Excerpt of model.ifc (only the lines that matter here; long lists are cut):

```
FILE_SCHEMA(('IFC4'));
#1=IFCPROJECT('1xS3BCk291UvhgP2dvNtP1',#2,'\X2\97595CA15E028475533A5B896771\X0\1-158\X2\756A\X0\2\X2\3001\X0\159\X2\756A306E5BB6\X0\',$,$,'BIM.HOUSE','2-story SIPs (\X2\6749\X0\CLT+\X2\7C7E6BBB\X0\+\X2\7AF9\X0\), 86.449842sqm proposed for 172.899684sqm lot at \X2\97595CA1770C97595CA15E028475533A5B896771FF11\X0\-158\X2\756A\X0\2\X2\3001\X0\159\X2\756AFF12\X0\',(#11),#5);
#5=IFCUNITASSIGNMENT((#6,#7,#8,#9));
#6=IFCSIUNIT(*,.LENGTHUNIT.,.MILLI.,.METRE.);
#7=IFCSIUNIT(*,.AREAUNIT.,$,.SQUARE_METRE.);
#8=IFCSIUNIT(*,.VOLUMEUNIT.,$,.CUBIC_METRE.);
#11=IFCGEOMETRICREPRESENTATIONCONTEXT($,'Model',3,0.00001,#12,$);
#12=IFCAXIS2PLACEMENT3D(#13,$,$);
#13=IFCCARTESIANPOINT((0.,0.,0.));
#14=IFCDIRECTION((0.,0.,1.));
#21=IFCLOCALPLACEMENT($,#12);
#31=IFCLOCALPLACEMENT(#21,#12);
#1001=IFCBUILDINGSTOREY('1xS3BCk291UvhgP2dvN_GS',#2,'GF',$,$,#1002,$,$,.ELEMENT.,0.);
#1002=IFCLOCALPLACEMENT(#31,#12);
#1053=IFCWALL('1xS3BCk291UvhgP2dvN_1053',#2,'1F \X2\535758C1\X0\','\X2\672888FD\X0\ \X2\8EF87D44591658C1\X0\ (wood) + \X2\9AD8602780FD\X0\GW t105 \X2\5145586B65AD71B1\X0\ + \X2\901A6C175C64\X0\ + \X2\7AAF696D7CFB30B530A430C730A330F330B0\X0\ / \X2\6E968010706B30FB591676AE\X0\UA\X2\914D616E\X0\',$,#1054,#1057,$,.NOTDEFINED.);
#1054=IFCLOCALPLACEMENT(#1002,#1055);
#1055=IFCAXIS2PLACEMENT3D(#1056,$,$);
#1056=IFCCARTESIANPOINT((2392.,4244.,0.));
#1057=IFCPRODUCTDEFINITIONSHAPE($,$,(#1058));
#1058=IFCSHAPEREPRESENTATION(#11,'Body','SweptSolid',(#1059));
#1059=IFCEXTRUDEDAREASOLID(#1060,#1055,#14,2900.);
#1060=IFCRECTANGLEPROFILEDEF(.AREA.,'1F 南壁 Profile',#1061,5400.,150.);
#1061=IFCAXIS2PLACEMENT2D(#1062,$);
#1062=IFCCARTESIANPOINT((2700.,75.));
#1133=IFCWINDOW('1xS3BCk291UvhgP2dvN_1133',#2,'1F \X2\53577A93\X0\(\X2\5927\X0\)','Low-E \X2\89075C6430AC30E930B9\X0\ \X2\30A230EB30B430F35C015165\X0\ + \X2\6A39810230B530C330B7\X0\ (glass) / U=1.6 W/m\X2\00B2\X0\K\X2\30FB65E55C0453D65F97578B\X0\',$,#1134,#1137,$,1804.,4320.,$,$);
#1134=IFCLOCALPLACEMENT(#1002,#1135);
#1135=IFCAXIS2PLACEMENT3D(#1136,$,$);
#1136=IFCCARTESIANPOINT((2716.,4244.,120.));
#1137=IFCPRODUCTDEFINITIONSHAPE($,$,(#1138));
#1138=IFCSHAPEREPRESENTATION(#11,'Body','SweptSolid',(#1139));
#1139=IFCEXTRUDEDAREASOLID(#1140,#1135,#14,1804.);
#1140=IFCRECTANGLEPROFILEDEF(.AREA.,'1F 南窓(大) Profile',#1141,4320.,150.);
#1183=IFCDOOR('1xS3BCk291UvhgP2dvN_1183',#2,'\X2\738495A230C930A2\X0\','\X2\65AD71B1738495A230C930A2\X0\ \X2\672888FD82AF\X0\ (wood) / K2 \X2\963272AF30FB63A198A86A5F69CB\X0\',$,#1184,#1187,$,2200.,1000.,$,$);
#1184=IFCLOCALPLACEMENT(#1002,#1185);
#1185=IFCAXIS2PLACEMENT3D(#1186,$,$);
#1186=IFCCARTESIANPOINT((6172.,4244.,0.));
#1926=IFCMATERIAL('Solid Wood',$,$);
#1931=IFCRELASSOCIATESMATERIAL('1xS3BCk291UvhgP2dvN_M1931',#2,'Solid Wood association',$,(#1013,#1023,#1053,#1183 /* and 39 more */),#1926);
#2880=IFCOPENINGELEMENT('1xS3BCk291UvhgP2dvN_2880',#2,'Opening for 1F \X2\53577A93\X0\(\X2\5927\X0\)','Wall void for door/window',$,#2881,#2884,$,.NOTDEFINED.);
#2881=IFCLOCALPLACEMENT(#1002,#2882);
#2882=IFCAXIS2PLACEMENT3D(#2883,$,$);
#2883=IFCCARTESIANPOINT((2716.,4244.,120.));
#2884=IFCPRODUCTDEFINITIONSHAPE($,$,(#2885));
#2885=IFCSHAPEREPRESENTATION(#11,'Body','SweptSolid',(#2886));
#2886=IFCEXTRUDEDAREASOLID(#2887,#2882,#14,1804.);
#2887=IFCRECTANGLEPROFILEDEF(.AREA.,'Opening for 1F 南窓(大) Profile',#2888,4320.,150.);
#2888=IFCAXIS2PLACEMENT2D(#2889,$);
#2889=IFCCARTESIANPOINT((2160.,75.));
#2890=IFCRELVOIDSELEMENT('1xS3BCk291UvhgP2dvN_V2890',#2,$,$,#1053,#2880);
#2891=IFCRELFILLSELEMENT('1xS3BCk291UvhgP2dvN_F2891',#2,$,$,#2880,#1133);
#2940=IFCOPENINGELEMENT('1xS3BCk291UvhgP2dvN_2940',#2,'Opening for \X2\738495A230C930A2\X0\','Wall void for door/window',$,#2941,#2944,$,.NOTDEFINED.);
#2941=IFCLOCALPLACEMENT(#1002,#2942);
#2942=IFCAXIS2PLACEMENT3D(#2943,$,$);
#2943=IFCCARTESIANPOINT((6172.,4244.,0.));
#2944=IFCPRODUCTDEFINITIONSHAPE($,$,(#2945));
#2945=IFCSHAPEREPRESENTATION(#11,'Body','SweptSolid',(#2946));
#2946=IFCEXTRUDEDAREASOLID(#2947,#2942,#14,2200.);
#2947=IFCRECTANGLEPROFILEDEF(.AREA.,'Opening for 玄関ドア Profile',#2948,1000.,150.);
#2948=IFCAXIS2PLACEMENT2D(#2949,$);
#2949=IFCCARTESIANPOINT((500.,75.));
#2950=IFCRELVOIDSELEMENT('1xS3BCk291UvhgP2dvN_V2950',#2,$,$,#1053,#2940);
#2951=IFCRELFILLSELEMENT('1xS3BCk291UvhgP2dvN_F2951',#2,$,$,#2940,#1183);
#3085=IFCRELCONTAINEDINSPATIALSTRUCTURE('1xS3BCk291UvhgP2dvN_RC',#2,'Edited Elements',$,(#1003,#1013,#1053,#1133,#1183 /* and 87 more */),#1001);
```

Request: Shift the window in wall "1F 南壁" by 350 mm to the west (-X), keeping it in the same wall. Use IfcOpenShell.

```python
import ifcopenshell
import ifcopenshell.api.geometry
import ifcopenshell.util.placement

model = ifcopenshell.open("model.ifc")

window = model.by_guid("1xS3BCk291UvhgP2dvN_1133")
opening = window.FillsVoids[0].RelatingOpeningElement
wall = opening.VoidsElements[0].RelatingBuildingElement

wall_matrix = ifcopenshell.util.placement.get_local_placement(wall.ObjectPlacement)
shift = wall_matrix[:3, 0] * -350.0
before = ifcopenshell.util.placement.get_local_placement(window.ObjectPlacement)[:3, 3].copy()

# The window is not placed relative to its opening, so move both.
for product in (opening, window):
    matrix = ifcopenshell.util.placement.get_local_placement(product.ObjectPlacement)
    matrix[:3, 3] += shift
    ifcopenshell.api.geometry.edit_object_placement(model, product=product, matrix=matrix, is_si=False)

after = ifcopenshell.util.placement.get_local_placement(window.ObjectPlacement)[:3, 3]
print("window moved by", (after - before).round(3) + 0.0)

model.write("model_updated.ifc")
```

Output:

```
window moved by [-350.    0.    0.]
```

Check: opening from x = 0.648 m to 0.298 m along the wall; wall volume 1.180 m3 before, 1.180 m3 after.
